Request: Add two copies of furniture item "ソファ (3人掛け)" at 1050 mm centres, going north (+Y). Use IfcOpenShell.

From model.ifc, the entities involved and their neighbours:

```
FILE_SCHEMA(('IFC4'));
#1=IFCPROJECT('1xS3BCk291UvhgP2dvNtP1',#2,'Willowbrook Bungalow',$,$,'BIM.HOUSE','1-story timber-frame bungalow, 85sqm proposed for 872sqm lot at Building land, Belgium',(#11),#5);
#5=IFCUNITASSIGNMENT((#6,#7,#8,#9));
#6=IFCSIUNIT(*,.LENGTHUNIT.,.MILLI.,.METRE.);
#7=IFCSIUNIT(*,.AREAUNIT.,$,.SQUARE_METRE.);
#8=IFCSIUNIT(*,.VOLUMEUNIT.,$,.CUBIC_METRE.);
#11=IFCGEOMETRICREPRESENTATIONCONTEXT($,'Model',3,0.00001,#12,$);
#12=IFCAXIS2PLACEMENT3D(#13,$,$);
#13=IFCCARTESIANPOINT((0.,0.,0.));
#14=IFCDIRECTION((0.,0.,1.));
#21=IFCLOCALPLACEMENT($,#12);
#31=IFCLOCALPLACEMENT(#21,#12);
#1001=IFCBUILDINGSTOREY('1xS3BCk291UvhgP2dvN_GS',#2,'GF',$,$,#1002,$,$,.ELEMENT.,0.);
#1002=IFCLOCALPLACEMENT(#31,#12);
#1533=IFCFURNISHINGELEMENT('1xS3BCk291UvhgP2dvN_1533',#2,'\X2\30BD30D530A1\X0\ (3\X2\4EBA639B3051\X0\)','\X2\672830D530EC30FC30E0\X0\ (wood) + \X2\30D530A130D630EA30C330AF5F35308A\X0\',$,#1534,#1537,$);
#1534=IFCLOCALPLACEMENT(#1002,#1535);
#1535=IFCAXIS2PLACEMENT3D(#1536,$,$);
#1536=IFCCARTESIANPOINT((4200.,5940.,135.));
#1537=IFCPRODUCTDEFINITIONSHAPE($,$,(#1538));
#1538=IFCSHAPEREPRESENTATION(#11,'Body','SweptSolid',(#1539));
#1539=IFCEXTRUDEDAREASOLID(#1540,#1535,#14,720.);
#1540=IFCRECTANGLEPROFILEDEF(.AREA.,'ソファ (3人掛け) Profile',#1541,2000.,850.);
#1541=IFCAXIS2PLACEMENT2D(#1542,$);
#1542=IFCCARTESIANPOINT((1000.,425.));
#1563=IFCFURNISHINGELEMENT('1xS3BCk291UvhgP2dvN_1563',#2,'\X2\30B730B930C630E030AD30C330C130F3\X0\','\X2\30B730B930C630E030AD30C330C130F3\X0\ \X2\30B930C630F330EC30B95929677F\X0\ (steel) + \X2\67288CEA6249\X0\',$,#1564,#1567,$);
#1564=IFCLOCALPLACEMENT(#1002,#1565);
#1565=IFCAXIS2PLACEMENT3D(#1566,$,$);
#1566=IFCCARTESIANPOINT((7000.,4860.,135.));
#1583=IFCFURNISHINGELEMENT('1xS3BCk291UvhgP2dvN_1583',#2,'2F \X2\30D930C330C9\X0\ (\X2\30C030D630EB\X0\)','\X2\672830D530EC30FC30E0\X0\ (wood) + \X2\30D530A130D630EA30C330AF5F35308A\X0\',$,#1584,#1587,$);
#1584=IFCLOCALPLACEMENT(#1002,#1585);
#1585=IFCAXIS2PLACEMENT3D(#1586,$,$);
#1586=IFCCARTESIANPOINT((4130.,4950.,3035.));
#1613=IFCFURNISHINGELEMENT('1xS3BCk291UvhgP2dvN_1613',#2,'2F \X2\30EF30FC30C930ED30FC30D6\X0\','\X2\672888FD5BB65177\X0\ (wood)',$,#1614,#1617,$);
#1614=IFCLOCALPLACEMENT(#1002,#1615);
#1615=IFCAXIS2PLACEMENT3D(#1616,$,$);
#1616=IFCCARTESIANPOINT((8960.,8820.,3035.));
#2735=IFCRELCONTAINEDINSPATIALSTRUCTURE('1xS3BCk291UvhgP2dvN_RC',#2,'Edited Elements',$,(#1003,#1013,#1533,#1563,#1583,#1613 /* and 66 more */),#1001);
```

```python
import numpy as np
import ifcopenshell
import ifcopenshell.api.geometry
import ifcopenshell.api.root
import ifcopenshell.util.element
import ifcopenshell.util.placement
import ifcopenshell.util.unit

model = ifcopenshell.open("model.ifc")
unit_scale = ifcopenshell.util.unit.calculate_unit_scale(model)


def reuse_history(source, copy):
    """copy_class also copies each property set's owner history, people and application; keep the originals."""
    for rel in copy.IsDefinedBy:
        if rel.is_a("IfcRelDefinesByProperties") and (history := rel.RelatingPropertyDefinition.OwnerHistory):
            rel.RelatingPropertyDefinition.OwnerHistory = source.OwnerHistory
            ifcopenshell.util.element.remove_deep2(model, history)


source = model.by_guid("1xS3BCk291UvhgP2dvN_1533")
base = ifcopenshell.util.placement.get_local_placement(source.ObjectPlacement)
step = np.array([0.0, 1.0, 0.0]) * 1.05 / unit_scale

for i in range(1, 3):
    copy = ifcopenshell.api.root.copy_class(model, product=source)
    copy.Representation = ifcopenshell.util.element.copy_deep(
        model, source.Representation, exclude=["IfcGeometricRepresentationContext", "IfcRepresentationMap"]
    )
    reuse_history(source, copy)
    matrix = base.copy()
    matrix[:3, 3] += i * step
    print("added at", matrix[:3, 3].round(3) + 0.0)
    ifcopenshell.api.geometry.edit_object_placement(model, product=copy, matrix=matrix, is_si=False)

model.write("model_v2.ifc")
```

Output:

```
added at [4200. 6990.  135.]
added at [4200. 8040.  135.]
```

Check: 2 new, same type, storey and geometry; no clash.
